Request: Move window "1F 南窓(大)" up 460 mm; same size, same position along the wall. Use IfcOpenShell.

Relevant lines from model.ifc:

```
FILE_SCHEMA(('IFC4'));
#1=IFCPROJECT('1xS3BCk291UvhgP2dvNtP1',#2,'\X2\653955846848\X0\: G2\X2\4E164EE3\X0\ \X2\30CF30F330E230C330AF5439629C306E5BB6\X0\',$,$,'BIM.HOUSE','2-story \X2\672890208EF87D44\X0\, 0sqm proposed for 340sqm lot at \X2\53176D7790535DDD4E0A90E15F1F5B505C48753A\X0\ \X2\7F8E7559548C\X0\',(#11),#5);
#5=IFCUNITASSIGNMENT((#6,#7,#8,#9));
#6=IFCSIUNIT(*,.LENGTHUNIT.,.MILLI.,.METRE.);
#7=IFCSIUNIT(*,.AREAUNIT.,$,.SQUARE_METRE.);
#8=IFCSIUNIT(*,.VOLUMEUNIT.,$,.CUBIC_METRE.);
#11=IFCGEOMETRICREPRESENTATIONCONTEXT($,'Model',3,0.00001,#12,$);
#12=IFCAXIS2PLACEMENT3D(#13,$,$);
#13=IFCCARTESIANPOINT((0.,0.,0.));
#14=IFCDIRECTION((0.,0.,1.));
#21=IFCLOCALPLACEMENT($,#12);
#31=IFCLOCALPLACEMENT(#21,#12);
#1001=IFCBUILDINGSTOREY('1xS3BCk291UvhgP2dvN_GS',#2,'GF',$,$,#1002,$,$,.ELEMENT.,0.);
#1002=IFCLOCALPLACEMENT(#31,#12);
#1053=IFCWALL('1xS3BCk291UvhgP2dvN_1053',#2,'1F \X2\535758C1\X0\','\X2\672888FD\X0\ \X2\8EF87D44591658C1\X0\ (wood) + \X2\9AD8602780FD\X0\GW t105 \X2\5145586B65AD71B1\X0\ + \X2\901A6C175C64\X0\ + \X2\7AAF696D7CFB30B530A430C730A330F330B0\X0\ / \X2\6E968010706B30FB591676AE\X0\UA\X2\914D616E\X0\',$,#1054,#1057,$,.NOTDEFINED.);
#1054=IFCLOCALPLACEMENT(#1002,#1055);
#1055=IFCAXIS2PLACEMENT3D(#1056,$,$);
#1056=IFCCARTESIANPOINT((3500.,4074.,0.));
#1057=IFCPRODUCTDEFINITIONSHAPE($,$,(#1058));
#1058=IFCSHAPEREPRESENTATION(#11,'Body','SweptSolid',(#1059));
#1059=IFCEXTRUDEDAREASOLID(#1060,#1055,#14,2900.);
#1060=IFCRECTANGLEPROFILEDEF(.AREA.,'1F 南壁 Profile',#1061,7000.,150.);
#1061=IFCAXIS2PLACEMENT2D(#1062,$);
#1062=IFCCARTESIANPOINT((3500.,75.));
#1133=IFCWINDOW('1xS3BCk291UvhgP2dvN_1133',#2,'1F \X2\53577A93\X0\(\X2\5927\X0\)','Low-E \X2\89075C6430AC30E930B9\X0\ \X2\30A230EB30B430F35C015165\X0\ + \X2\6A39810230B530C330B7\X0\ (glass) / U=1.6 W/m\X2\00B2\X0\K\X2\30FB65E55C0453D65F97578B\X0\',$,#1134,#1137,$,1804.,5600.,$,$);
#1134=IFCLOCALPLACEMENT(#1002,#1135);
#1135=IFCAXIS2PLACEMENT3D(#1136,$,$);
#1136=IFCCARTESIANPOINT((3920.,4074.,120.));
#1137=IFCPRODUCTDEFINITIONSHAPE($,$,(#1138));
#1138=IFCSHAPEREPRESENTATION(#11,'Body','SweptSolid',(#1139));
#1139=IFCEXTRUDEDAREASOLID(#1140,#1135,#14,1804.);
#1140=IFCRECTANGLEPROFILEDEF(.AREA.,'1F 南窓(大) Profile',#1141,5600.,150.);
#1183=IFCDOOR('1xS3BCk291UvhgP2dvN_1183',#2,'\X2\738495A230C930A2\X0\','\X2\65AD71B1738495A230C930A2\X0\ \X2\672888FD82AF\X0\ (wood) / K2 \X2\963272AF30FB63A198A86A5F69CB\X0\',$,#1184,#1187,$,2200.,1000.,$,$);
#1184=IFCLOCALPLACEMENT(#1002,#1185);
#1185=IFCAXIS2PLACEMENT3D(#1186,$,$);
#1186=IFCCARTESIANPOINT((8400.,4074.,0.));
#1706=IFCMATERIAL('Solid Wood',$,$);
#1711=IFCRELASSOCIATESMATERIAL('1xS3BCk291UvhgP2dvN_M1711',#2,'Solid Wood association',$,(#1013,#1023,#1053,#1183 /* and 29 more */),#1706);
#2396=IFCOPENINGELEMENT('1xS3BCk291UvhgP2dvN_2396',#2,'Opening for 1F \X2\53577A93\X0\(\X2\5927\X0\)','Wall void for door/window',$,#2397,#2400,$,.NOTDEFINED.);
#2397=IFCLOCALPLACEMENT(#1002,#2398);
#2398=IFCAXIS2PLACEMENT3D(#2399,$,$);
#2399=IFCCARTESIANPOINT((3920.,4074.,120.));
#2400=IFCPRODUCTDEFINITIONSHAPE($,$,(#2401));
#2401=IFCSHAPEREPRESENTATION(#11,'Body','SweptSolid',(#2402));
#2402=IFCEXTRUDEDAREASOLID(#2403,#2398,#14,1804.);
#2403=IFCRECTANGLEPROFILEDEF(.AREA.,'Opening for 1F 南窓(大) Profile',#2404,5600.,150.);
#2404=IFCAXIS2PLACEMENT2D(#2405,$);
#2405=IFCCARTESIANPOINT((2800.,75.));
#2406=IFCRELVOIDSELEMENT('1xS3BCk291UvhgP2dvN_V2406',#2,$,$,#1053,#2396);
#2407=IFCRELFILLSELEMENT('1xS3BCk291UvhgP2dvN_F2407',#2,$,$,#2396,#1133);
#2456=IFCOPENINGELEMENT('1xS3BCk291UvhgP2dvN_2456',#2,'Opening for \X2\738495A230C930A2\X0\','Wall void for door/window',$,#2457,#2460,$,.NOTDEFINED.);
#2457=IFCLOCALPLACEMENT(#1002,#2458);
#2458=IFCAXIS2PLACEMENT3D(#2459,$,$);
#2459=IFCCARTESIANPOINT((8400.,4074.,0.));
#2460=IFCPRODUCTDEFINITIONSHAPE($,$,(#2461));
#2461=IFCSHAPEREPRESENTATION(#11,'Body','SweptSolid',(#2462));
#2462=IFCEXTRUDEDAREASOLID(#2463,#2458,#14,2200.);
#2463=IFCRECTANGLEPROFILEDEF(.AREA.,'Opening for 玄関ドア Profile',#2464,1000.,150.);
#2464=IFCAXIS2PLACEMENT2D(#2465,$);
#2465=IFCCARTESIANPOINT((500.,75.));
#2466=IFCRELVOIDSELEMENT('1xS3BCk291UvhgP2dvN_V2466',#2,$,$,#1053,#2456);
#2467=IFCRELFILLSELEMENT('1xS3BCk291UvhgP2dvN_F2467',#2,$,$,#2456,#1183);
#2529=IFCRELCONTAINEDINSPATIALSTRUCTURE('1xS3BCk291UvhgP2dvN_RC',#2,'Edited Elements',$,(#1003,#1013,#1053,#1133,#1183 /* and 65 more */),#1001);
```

```python
import numpy as np
import ifcopenshell
import ifcopenshell.api.geometry
import ifcopenshell.util.placement
import ifcopenshell.util.unit

model = ifcopenshell.open("model.ifc")
unit_scale = ifcopenshell.util.unit.calculate_unit_scale(model)

window = model.by_id(1133)
opening = window.FillsVoids[0].RelatingOpeningElement
dz = 460.0

shift = np.array([0.0, 0.0, dz])
# The window is not placed relative to its opening, so move both.
for product in (opening, window):
    matrix = ifcopenshell.util.placement.get_local_placement(product.ObjectPlacement)
    matrix[:3, 3] += shift
    ifcopenshell.api.geometry.edit_object_placement(model, product=product, matrix=matrix, is_si=False)

print(f"moved by {dz * unit_scale:+.3f} m")

model.write("model_v2.ifc")
```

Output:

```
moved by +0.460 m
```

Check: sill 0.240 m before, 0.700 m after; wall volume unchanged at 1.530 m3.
